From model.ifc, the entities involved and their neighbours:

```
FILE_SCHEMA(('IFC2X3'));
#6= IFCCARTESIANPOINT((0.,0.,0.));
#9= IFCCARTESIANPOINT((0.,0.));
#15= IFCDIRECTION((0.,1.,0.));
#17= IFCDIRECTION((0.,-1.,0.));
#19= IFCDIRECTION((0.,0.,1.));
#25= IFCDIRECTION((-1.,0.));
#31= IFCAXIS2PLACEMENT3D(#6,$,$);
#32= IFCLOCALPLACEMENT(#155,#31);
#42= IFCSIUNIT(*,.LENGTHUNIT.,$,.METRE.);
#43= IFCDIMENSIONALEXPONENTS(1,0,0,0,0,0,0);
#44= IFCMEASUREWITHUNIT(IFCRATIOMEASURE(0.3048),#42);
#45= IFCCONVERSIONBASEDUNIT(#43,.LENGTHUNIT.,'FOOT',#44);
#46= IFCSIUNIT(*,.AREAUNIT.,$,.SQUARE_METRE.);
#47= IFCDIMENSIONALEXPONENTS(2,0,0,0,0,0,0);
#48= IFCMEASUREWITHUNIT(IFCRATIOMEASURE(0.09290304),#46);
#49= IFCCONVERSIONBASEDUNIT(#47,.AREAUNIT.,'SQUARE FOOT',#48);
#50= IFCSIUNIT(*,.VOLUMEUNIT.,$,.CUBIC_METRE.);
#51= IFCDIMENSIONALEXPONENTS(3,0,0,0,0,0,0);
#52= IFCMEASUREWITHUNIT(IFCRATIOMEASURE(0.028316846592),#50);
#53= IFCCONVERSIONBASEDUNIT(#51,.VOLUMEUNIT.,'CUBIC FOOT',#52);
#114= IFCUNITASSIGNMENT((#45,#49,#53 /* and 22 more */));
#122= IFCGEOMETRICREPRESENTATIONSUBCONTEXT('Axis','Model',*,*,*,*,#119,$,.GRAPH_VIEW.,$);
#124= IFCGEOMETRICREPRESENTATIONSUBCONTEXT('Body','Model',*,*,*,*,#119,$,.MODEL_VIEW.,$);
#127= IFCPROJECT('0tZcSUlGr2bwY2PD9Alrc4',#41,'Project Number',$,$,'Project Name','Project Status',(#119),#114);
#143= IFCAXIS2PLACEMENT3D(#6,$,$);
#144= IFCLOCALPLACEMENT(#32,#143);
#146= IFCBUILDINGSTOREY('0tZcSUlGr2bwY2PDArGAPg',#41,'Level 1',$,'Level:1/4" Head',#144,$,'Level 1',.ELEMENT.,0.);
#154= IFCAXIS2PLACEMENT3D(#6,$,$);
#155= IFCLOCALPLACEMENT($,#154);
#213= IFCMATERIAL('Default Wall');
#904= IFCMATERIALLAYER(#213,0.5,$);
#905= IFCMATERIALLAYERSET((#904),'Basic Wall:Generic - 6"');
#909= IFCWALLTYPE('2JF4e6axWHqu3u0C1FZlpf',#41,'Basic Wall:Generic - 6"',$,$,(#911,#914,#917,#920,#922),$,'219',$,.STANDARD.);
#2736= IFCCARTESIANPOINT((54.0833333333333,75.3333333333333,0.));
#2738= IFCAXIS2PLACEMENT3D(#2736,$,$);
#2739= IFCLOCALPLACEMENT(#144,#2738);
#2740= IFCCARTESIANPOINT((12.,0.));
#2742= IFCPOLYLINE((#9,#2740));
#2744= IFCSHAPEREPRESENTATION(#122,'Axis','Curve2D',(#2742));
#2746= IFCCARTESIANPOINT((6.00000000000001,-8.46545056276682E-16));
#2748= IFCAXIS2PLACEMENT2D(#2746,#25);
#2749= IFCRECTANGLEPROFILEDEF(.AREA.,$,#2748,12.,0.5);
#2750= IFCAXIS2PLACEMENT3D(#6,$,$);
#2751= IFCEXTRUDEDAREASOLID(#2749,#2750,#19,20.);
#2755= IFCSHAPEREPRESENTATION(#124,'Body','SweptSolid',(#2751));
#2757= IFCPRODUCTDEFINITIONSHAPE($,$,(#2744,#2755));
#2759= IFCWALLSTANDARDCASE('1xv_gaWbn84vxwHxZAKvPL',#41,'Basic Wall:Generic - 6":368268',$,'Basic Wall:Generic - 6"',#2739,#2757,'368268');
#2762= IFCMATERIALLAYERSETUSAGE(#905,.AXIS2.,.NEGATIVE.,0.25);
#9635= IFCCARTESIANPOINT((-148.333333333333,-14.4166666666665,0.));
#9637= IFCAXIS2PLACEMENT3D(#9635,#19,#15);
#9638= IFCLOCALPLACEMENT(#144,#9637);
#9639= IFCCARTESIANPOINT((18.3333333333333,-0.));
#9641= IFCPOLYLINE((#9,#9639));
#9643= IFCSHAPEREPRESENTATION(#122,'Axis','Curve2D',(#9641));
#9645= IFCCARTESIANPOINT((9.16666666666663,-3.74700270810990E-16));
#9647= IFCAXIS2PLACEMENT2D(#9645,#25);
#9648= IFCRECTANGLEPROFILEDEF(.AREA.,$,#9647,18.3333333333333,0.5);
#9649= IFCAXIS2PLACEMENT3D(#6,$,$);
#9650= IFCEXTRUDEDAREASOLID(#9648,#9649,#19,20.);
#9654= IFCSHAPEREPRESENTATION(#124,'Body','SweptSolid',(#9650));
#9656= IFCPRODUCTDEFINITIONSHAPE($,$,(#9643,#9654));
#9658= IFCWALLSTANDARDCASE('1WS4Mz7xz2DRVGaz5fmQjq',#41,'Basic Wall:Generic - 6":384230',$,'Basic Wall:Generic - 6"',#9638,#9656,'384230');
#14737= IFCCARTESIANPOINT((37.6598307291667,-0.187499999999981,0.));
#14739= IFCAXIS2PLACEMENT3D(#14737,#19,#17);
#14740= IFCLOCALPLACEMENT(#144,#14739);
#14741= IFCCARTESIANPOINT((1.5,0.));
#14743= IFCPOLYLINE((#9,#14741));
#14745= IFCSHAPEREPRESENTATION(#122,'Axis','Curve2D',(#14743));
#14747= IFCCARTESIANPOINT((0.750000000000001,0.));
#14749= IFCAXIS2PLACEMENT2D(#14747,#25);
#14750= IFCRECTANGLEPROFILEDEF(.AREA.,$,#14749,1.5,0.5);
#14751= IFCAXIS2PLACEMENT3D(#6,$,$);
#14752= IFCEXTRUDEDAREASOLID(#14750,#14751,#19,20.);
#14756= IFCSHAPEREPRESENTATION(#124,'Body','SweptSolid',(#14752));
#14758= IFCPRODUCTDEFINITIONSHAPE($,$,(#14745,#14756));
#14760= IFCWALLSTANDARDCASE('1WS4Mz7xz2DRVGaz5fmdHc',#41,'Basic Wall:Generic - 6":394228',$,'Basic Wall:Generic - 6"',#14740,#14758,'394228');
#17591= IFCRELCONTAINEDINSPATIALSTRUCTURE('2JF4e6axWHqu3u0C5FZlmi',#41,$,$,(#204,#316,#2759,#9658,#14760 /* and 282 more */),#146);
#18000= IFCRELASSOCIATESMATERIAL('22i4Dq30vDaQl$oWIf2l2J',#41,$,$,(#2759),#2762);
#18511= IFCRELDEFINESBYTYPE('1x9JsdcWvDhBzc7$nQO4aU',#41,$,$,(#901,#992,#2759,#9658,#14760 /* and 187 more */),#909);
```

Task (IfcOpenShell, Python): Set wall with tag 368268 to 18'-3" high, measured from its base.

```python
import ifcopenshell
import ifcopenshell.geom
import ifcopenshell.util.representation
import ifcopenshell.util.shape
import ifcopenshell.util.unit

model = ifcopenshell.open("model.ifc")
unit_scale = ifcopenshell.util.unit.calculate_unit_scale(model)
settings = ifcopenshell.geom.settings()


def volume(element):
    """Net volume in cubic metres, openings subtracted."""
    shape = ifcopenshell.geom.create_shape(settings, element)
    return ifcopenshell.util.shape.get_volume(shape.geometry)


wall = model.by_guid("1xv_gaWbn84vxwHxZAKvPL")
before = volume(wall)

body = ifcopenshell.util.representation.get_representation(wall, "Model", "Body")
solid = body.Items[0]
old_height = solid.Depth
solid.Depth = 219 * 0.0254 / unit_scale
after = volume(wall)

print(f"height {old_height:g} -> {solid.Depth:g}, volume {before:.3f} -> {after:.3f} m3")

model.write("model_v2.ifc")
```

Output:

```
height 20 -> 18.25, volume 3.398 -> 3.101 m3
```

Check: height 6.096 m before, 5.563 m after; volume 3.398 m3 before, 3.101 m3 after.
